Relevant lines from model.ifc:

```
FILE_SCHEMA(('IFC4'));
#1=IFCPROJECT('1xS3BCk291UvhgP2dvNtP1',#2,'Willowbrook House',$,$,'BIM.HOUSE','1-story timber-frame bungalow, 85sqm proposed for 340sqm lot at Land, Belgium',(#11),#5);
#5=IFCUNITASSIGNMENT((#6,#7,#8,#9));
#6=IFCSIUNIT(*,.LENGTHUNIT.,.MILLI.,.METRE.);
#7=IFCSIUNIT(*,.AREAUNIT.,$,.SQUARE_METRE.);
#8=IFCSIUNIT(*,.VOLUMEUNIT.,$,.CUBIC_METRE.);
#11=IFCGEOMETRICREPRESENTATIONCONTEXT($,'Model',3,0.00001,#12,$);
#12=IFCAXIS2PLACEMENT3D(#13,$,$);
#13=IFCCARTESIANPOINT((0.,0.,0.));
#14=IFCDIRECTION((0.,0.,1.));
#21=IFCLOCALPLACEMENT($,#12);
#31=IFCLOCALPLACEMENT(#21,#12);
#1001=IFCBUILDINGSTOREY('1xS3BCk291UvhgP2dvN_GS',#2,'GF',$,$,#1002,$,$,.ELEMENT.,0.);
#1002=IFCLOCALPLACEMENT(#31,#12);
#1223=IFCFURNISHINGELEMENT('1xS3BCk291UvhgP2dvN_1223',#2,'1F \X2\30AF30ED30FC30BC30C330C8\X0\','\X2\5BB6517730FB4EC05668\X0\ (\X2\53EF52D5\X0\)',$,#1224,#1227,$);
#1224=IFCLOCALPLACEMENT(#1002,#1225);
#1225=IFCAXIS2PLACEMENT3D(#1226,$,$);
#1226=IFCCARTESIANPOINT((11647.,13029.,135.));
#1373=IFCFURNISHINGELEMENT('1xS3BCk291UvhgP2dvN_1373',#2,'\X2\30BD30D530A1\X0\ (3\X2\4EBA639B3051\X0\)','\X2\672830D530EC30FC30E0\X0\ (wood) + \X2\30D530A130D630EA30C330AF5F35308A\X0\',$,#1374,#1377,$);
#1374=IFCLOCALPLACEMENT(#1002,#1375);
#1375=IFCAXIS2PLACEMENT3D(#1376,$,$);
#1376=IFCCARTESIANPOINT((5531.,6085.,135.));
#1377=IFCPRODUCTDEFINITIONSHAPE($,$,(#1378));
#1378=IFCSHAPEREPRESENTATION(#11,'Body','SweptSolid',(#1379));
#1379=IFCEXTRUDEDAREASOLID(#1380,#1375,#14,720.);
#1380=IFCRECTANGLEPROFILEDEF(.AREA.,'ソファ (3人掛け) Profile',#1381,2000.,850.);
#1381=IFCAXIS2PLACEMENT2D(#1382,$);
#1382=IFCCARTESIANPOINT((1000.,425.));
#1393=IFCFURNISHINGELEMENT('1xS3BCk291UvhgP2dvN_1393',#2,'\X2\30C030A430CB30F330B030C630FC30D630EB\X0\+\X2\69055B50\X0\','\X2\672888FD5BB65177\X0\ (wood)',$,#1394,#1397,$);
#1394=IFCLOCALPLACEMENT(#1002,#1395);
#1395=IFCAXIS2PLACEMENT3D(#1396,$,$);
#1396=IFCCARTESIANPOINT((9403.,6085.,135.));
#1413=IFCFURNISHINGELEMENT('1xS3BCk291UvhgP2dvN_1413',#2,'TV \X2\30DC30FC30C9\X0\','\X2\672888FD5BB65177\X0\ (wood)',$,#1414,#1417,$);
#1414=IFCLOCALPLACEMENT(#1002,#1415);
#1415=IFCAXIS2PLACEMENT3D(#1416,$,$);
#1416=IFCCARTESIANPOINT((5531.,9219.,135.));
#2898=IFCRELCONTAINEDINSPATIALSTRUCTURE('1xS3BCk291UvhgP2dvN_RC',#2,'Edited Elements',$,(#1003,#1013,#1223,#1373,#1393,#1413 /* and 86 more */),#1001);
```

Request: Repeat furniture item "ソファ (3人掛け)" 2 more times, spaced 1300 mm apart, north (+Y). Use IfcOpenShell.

```python
import numpy as np
import ifcopenshell
import ifcopenshell.api.geometry
import ifcopenshell.api.root
import ifcopenshell.util.element
import ifcopenshell.util.placement

model = ifcopenshell.open("model.ifc")


def reuse_history(source, copy):
    """copy_class also copies each property set's owner history, people and application; keep the originals."""
    for rel in copy.IsDefinedBy:
        if rel.is_a("IfcRelDefinesByProperties") and (history := rel.RelatingPropertyDefinition.OwnerHistory):
            rel.RelatingPropertyDefinition.OwnerHistory = source.OwnerHistory
            ifcopenshell.util.element.remove_deep2(model, history)


source = model.by_guid("1xS3BCk291UvhgP2dvN_1373")
base = ifcopenshell.util.placement.get_local_placement(source.ObjectPlacement)
step = np.array([0.0, 1.0, 0.0]) * 1300.0

for i in range(1, 3):
    copy = ifcopenshell.api.root.copy_class(model, product=source)
    copy.Representation = ifcopenshell.util.element.copy_deep(
        model, source.Representation, exclude=["IfcGeometricRepresentationContext", "IfcRepresentationMap"]
    )
    reuse_history(source, copy)
    matrix = base.copy()
    matrix[:3, 3] += i * step
    print("added at", matrix[:3, 3].round(3) + 0.0)
    ifcopenshell.api.geometry.edit_object_placement(model, product=copy, matrix=matrix, is_si=False)

model.write("model_rev.ifc")
```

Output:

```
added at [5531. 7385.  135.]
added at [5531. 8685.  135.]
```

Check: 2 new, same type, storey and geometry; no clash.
